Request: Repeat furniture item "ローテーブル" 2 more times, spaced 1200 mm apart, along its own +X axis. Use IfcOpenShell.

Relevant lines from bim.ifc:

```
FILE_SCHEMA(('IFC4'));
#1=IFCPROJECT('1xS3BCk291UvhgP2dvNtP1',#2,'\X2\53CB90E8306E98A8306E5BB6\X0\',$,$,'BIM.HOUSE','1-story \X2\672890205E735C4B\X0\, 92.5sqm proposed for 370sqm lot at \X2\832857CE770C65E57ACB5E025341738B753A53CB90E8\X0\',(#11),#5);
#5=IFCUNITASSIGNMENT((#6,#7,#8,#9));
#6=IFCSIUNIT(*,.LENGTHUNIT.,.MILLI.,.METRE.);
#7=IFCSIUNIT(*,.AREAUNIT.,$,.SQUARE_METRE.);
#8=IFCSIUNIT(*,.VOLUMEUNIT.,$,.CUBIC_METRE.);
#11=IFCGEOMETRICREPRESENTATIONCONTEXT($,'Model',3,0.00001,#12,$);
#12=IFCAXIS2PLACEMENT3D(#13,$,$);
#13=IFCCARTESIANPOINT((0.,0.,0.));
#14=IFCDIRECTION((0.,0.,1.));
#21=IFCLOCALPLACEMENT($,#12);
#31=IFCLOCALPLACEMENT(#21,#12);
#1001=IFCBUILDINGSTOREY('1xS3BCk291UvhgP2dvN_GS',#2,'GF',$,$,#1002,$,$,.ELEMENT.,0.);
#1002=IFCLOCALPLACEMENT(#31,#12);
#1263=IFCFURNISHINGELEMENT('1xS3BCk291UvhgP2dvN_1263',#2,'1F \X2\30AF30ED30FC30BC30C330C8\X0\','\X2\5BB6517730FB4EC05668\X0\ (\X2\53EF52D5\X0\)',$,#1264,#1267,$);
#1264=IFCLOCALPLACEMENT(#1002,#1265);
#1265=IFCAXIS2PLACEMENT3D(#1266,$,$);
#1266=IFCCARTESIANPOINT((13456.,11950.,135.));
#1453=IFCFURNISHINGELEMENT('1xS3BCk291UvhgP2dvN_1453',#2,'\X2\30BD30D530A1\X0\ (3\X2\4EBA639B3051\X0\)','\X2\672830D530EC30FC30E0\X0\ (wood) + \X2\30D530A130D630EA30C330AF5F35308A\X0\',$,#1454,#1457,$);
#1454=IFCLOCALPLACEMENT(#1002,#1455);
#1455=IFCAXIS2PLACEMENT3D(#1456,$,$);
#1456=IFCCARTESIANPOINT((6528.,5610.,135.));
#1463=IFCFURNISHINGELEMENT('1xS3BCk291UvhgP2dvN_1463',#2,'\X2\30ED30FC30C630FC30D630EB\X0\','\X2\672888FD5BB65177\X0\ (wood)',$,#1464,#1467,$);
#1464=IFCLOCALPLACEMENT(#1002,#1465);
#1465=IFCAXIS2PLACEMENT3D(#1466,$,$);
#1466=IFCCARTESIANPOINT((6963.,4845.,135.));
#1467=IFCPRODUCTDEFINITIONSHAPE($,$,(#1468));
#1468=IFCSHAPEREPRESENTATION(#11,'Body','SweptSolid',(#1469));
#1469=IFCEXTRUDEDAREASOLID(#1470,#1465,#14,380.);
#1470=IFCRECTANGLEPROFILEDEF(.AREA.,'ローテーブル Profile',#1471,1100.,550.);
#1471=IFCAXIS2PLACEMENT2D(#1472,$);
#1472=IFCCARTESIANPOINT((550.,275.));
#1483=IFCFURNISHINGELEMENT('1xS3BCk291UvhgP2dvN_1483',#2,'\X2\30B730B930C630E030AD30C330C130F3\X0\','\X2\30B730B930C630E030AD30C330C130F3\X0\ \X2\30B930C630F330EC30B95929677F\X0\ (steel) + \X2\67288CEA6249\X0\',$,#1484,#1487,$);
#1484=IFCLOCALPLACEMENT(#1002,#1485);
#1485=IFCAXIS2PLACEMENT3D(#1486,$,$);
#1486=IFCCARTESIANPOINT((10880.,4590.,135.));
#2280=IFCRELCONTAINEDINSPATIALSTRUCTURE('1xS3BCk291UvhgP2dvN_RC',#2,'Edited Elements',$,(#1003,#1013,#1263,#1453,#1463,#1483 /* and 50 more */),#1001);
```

```python
import ifcopenshell
import ifcopenshell.api.geometry
import ifcopenshell.api.root
import ifcopenshell.util.element
import ifcopenshell.util.placement
import ifcopenshell.util.unit

model = ifcopenshell.open("bim.ifc")
unit_scale = ifcopenshell.util.unit.calculate_unit_scale(model)


def reuse_history(source, copy):
    """copy_class also copies each property set's owner history, people and application; keep the originals."""
    for rel in copy.IsDefinedBy:
        if rel.is_a("IfcRelDefinesByProperties") and (history := rel.RelatingPropertyDefinition.OwnerHistory):
            rel.RelatingPropertyDefinition.OwnerHistory = source.OwnerHistory
            ifcopenshell.util.element.remove_deep2(model, history)


source = model.by_id(1463)
base = ifcopenshell.util.placement.get_local_placement(source.ObjectPlacement)
step = base[:3, 0] * 1.2 / unit_scale

for i in range(1, 3):
    copy = ifcopenshell.api.root.copy_class(model, product=source)
    copy.Representation = ifcopenshell.util.element.copy_deep(
        model, source.Representation, exclude=["IfcGeometricRepresentationContext", "IfcRepresentationMap"]
    )
    reuse_history(source, copy)
    matrix = base.copy()
    matrix[:3, 3] += i * step
    print("added at", matrix[:3, 3].round(3) + 0.0)
    ifcopenshell.api.geometry.edit_object_placement(model, product=copy, matrix=matrix, is_si=False)

model.write("bim-out.ifc")
```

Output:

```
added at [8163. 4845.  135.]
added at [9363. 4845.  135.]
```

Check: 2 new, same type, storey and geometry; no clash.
